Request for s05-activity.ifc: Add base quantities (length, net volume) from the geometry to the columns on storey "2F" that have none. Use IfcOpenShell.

First a look at what the model holds.

```python
import ifcopenshell
import ifcopenshell.util.element
import ifcopenshell.util.unit

model = ifcopenshell.open("s05-activity.ifc")
print(model.schema)
for unit_type in ("LENGTHUNIT", "AREAUNIT", "VOLUMEUNIT"):
    print(unit_type, ifcopenshell.util.unit.calculate_unit_scale(model, unit_type))
storey = next(s for s in model.by_type("IfcBuildingStorey") if s.Name == "2F")
columns = [e for e in ifcopenshell.util.element.get_decomposition(storey) if e.is_a("IfcColumn")]
for e in sorted(columns, key=lambda e: e.id()):
    print(e.id(), e.is_a(), e.Name, list(ifcopenshell.util.element.get_psets(e, qtos_only=True)), sep=" | ")
```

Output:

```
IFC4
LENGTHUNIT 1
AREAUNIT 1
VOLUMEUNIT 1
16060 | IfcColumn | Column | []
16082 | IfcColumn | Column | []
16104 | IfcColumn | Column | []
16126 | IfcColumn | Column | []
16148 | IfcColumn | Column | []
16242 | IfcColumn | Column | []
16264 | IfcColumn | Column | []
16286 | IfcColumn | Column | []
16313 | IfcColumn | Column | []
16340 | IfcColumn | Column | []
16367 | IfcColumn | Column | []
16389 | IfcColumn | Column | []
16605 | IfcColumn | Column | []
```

```python
import ifcopenshell
import ifcopenshell.api.pset
import ifcopenshell.geom
import ifcopenshell.util.element
import ifcopenshell.util.shape
import ifcopenshell.util.unit

model = ifcopenshell.open("s05-activity.ifc")
unit_scale = ifcopenshell.util.unit.calculate_unit_scale(model)
volume_scale = ifcopenshell.util.unit.calculate_unit_scale(model, "VOLUMEUNIT")
settings = ifcopenshell.geom.settings()

storey = next(s for s in model.by_type("IfcBuildingStorey") if s.Name == "2F")
columns = [e for e in ifcopenshell.util.element.get_decomposition(storey) if e.is_a("IfcColumn")]

for e in sorted(columns, key=lambda e: e.id()):
    if ifcopenshell.util.element.get_psets(e, qtos_only=True, should_inherit=False):
        continue
    # Geometry comes back in metres, in the element's own axes.
    shape = ifcopenshell.geom.create_shape(settings, e)
    values = {
        "Length": ifcopenshell.util.shape.get_z(shape.geometry) / unit_scale,
        "NetVolume": ifcopenshell.util.shape.get_volume(shape.geometry) / volume_scale,
    }
    qto = ifcopenshell.api.pset.add_qto(model, product=e, name="Qto_ColumnBaseQuantities")
    ifcopenshell.api.pset.edit_qto(model, qto=qto, properties=values)
    print(e.id(), {k: round(v, 3) for k, v in values.items()})

model.write("s05-activity_updated.ifc")
```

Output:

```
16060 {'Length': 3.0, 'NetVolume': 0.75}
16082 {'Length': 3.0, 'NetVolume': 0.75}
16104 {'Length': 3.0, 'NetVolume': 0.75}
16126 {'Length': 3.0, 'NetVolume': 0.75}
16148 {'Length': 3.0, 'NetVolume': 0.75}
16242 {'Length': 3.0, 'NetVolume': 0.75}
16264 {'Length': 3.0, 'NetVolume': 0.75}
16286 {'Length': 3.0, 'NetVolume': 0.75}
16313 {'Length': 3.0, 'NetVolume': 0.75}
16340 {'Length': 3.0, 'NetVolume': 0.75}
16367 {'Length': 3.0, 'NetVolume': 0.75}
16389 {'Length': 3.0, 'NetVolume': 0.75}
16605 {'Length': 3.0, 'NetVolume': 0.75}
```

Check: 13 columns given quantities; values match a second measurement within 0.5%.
